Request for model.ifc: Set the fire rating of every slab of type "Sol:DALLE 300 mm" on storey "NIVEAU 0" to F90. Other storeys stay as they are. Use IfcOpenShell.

First a look at what the model holds.

```python
import ifcopenshell
import ifcopenshell.util.element

model = ifcopenshell.open("model.ifc")
print(model.schema)
storey = next(s for s in model.by_type("IfcBuildingStorey") if s.Name == "NIVEAU 0")
slabs = [e for e in ifcopenshell.util.element.get_decomposition(storey) if e.is_a("IfcSlab")]
seen = {}
for e in slabs:
    element_type = ifcopenshell.util.element.get_type(e)
    key = (element_type.Name if element_type != e and element_type else None, ifcopenshell.util.element.get_pset(e, "Pset_SlabCommon", "FireRating"))
    seen[key] = seen.get(key, 0) + 1
for (name, value), count in sorted(seen.items(), key=str):
    print(count, "x", name, "|", value)
```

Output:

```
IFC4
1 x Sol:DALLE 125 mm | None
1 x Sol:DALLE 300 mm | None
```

```python
import ifcopenshell
import ifcopenshell.api.pset
import ifcopenshell.util.element

model = ifcopenshell.open("model.ifc")

storey = next(s for s in model.by_type("IfcBuildingStorey") if s.Name == "NIVEAU 0")
slabs = [e for e in ifcopenshell.util.element.get_decomposition(storey) if e.is_a("IfcSlab")]

count = 0
for e in slabs:
    element_type = ifcopenshell.util.element.get_type(e)
    if element_type in (None, e) or element_type.Name != "Sol:DALLE 300 mm":
        continue
    # add_pset returns the element's existing set when there is one.
    pset = ifcopenshell.api.pset.add_pset(model, product=e, name="Pset_SlabCommon")
    ifcopenshell.api.pset.edit_pset(model, pset=pset, properties={"FireRating": "F90"})
    count += 1

print(count, "slabs updated")

model.write("model-out.ifc")
```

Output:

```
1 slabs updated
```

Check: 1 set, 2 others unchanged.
